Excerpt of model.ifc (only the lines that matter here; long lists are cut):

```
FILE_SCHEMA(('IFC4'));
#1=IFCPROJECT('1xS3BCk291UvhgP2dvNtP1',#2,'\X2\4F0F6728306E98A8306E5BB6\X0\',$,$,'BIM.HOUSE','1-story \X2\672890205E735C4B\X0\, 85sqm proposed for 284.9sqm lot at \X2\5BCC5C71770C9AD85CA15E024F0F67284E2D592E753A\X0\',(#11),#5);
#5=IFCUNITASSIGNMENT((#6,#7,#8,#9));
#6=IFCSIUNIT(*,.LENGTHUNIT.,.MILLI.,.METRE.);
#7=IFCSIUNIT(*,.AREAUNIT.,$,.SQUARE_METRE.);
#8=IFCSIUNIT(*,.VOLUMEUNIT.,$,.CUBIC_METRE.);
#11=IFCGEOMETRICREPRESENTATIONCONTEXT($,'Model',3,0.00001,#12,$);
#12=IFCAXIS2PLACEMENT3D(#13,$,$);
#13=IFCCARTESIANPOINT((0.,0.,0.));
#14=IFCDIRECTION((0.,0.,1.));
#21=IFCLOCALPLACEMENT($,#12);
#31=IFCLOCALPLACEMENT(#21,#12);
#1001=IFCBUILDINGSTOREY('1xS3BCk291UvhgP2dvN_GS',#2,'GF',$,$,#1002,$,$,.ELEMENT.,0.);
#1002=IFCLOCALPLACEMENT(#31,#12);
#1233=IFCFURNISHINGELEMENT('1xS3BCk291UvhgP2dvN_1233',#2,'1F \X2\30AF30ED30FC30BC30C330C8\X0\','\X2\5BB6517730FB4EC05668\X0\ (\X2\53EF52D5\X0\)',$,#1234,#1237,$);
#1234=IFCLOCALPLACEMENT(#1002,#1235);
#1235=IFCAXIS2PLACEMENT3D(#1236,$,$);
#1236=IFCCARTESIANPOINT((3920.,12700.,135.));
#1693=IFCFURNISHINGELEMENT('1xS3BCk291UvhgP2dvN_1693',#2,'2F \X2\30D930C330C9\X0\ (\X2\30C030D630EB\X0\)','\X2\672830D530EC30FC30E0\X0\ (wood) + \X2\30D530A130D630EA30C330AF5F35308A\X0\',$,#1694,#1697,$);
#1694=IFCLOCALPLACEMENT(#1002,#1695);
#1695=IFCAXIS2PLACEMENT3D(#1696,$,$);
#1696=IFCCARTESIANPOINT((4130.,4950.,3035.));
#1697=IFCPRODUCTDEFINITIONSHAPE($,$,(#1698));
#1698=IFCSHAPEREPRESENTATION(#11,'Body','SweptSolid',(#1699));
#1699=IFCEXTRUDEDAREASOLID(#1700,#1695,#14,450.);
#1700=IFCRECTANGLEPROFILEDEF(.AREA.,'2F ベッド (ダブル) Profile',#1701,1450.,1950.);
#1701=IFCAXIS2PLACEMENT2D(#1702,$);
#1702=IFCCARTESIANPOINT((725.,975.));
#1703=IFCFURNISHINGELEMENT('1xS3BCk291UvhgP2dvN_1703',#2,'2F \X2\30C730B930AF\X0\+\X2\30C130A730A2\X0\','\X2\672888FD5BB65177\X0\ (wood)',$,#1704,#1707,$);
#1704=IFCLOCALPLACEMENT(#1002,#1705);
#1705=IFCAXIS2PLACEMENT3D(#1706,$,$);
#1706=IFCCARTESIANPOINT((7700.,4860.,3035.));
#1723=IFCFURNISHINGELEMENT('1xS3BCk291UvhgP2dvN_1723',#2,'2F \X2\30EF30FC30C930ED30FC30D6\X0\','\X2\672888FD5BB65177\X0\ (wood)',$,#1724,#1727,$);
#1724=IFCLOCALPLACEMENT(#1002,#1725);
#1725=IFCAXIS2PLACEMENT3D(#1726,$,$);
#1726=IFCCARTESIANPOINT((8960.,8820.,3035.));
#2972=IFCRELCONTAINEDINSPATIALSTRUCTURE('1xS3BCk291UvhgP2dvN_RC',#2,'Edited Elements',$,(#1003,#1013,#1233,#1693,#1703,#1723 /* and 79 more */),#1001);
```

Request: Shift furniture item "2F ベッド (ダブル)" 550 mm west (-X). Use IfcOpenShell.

```python
import ifcopenshell
import ifcopenshell.api.geometry
import ifcopenshell.util.placement

model = ifcopenshell.open("model.ifc")

item = model.by_guid("1xS3BCk291UvhgP2dvN_1693")
matrix = ifcopenshell.util.placement.get_local_placement(item.ObjectPlacement)
matrix[0, 3] -= 550.0
ifcopenshell.api.geometry.edit_object_placement(model, product=item, matrix=matrix, is_si=False)

print(ifcopenshell.util.placement.get_local_placement(item.ObjectPlacement).round(3) + 0.0)

model.write("model_rev.ifc")
```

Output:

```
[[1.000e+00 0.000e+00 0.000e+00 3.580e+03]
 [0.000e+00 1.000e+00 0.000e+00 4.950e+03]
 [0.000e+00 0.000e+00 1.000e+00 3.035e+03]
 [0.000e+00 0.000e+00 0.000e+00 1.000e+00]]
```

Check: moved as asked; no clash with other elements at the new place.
